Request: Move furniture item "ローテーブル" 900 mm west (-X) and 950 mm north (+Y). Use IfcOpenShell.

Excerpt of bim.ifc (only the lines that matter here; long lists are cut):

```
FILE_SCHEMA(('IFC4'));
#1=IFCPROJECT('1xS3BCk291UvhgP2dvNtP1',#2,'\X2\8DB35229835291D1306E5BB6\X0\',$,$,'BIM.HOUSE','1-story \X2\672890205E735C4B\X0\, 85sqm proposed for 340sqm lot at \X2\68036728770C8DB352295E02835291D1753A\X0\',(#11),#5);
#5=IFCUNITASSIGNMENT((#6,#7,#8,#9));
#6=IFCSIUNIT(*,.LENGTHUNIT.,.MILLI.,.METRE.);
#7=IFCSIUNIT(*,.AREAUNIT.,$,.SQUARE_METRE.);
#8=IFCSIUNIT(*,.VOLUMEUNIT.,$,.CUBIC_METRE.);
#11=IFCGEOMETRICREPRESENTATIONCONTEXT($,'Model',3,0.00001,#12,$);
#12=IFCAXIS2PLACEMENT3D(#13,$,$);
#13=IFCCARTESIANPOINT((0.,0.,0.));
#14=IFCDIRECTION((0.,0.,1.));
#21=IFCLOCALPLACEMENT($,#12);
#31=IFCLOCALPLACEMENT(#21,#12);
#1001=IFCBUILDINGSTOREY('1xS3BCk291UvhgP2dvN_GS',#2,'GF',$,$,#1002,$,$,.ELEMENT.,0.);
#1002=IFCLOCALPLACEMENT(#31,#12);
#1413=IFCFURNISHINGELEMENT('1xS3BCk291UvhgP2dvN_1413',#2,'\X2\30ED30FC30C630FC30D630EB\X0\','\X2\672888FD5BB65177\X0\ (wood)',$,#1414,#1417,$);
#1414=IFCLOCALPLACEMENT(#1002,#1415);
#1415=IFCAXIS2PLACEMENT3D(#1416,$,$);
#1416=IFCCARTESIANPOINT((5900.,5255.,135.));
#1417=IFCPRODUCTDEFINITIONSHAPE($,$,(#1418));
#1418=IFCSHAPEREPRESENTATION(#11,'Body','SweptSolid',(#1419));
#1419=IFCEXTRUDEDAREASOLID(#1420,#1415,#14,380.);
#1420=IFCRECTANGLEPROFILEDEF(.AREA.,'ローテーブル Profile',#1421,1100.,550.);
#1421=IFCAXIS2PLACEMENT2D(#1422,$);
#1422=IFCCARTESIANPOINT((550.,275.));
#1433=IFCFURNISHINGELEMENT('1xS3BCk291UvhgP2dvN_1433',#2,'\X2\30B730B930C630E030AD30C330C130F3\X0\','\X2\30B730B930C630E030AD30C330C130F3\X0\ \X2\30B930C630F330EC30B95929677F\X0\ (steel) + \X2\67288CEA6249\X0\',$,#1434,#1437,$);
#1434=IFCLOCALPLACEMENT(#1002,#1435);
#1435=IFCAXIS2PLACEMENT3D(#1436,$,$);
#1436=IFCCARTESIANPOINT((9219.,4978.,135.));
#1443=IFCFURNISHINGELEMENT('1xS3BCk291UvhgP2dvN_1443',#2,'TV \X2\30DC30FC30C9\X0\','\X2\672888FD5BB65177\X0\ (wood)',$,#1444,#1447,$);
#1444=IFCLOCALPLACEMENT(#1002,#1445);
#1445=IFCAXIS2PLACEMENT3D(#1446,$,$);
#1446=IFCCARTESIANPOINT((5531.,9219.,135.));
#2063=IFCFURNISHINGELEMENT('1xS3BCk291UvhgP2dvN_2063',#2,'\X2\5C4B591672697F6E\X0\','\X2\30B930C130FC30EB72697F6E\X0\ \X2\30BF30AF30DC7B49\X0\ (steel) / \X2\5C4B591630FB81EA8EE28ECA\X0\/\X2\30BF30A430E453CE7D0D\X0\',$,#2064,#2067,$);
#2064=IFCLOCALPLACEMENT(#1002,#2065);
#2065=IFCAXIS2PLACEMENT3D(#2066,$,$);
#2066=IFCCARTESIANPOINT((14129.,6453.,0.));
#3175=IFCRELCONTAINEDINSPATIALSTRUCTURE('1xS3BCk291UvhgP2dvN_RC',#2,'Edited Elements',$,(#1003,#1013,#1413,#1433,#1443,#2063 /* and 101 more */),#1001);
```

```python
import ifcopenshell
import ifcopenshell.api.geometry
import ifcopenshell.util.placement

model = ifcopenshell.open("bim.ifc")

item = model.by_guid("1xS3BCk291UvhgP2dvN_1413")
matrix = ifcopenshell.util.placement.get_local_placement(item.ObjectPlacement)
matrix[0, 3] -= 900.0
matrix[1, 3] += 950.0
ifcopenshell.api.geometry.edit_object_placement(model, product=item, matrix=matrix, is_si=False)

print(ifcopenshell.util.placement.get_local_placement(item.ObjectPlacement).round(3) + 0.0)

model.write("bim_v2.ifc")
```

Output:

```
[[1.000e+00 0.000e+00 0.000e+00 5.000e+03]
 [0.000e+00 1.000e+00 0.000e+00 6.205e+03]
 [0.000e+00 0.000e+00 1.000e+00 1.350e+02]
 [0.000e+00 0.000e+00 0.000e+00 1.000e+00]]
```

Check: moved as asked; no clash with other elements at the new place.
